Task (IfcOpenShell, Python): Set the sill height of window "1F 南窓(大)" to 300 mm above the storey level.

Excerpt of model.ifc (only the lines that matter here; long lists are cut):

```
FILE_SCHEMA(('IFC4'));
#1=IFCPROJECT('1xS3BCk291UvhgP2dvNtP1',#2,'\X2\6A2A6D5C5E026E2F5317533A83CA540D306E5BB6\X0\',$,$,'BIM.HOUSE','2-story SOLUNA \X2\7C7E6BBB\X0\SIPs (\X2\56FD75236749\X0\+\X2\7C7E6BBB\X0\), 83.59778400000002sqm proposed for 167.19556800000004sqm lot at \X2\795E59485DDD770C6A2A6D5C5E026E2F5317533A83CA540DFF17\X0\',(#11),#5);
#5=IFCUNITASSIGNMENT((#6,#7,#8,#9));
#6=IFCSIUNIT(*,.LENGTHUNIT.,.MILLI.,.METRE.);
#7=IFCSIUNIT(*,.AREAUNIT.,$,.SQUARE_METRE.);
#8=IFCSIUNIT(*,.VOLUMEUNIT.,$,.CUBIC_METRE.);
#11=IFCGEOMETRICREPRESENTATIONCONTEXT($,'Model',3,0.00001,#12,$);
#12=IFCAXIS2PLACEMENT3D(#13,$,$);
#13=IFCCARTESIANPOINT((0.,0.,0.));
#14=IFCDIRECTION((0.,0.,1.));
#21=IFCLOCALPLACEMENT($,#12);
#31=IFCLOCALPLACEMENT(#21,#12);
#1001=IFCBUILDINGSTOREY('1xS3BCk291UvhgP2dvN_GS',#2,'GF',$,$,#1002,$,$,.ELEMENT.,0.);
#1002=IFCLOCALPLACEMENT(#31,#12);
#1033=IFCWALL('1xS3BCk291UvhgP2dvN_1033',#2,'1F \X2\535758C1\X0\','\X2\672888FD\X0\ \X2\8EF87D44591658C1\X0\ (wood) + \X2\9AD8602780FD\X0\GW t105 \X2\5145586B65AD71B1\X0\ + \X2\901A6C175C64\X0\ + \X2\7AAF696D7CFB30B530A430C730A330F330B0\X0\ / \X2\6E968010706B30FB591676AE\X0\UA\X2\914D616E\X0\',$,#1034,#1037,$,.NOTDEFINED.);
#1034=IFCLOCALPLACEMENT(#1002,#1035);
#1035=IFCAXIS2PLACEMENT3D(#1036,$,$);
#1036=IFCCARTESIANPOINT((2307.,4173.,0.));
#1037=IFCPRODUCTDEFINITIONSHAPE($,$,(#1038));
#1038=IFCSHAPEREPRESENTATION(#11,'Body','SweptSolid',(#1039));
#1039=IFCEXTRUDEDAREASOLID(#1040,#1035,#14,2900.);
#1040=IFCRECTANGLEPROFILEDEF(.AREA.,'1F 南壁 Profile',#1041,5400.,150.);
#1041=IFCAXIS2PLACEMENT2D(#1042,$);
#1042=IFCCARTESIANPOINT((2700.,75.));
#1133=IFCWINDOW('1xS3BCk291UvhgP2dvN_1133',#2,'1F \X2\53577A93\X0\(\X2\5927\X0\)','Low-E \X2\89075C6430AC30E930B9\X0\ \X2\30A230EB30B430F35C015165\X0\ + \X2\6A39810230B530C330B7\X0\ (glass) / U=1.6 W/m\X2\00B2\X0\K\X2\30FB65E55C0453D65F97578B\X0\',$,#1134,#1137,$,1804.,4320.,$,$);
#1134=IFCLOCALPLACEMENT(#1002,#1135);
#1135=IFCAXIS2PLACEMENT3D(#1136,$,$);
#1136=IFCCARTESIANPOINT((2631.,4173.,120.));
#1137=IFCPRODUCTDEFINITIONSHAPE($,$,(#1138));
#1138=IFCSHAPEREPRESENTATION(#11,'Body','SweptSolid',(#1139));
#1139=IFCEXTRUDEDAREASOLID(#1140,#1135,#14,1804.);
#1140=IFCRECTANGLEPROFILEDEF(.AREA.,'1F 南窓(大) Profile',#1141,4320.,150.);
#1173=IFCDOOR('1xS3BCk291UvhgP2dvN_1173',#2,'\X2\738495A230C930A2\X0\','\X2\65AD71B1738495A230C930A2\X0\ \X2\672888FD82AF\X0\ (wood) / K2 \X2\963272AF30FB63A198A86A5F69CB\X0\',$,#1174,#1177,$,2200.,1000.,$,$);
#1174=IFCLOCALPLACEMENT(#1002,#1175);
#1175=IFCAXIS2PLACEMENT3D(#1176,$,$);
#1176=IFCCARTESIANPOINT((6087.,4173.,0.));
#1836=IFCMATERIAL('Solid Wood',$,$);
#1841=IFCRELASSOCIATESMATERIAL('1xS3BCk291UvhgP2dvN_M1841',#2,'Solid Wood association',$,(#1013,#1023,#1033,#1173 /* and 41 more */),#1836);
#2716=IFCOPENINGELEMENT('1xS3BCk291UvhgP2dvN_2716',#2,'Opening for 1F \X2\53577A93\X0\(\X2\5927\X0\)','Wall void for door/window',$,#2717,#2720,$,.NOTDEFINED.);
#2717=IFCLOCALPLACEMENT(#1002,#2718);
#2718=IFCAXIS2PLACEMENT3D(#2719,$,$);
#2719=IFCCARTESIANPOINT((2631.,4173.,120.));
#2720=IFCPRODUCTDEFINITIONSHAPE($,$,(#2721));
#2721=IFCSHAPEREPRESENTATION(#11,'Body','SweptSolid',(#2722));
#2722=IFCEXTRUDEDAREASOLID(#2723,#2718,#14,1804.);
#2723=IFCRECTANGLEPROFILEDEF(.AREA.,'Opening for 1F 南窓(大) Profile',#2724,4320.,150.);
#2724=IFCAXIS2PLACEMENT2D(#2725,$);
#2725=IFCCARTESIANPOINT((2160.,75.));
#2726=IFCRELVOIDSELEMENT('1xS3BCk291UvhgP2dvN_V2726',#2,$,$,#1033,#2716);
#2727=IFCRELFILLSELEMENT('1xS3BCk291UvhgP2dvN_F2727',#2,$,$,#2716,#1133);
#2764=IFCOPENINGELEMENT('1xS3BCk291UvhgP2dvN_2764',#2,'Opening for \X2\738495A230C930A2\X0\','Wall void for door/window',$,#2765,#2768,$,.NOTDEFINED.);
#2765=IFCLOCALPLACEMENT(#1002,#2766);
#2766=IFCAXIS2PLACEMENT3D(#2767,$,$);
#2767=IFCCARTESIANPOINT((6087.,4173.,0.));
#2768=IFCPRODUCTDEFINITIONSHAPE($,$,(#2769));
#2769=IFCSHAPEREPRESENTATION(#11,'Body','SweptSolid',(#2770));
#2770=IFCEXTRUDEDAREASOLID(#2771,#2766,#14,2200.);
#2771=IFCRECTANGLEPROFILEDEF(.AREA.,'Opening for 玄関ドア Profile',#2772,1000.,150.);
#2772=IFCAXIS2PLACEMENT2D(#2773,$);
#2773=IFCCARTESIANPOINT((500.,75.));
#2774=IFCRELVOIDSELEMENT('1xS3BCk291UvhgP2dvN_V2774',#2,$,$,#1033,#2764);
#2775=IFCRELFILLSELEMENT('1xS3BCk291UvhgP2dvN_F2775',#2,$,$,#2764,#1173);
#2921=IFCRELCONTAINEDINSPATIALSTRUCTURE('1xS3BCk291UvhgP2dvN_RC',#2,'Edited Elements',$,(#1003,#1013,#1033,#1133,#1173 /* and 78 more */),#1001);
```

```python
import numpy as np
import ifcopenshell
import ifcopenshell.api.geometry
import ifcopenshell.geom
import ifcopenshell.util.element
import ifcopenshell.util.placement
import ifcopenshell.util.shape
import ifcopenshell.util.unit

model = ifcopenshell.open("model.ifc")
unit_scale = ifcopenshell.util.unit.calculate_unit_scale(model)

window = model.by_id(1133)
opening = window.FillsVoids[0].RelatingOpeningElement
storey = ifcopenshell.util.element.get_container(window, ifc_class="IfcBuildingStorey")
level = ifcopenshell.util.placement.get_local_placement(storey.ObjectPlacement)[2, 3]

# The opening's origin need not be at the sill, so measure its lowest point.
shape = ifcopenshell.geom.create_shape(ifcopenshell.geom.settings(), opening)
bottom = ifcopenshell.util.shape.get_shape_bottom_elevation(shape, shape.geometry) / unit_scale
dz = level + 300.0 - bottom

shift = np.array([0.0, 0.0, dz])
# The window is not placed relative to its opening, so move both.
for product in (opening, window):
    matrix = ifcopenshell.util.placement.get_local_placement(product.ObjectPlacement)
    matrix[:3, 3] += shift
    ifcopenshell.api.geometry.edit_object_placement(model, product=product, matrix=matrix, is_si=False)

print(f"moved by {dz * unit_scale:+.3f} m")

model.write("model_v2.ifc")
```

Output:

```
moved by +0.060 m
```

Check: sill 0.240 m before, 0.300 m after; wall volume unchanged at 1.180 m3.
